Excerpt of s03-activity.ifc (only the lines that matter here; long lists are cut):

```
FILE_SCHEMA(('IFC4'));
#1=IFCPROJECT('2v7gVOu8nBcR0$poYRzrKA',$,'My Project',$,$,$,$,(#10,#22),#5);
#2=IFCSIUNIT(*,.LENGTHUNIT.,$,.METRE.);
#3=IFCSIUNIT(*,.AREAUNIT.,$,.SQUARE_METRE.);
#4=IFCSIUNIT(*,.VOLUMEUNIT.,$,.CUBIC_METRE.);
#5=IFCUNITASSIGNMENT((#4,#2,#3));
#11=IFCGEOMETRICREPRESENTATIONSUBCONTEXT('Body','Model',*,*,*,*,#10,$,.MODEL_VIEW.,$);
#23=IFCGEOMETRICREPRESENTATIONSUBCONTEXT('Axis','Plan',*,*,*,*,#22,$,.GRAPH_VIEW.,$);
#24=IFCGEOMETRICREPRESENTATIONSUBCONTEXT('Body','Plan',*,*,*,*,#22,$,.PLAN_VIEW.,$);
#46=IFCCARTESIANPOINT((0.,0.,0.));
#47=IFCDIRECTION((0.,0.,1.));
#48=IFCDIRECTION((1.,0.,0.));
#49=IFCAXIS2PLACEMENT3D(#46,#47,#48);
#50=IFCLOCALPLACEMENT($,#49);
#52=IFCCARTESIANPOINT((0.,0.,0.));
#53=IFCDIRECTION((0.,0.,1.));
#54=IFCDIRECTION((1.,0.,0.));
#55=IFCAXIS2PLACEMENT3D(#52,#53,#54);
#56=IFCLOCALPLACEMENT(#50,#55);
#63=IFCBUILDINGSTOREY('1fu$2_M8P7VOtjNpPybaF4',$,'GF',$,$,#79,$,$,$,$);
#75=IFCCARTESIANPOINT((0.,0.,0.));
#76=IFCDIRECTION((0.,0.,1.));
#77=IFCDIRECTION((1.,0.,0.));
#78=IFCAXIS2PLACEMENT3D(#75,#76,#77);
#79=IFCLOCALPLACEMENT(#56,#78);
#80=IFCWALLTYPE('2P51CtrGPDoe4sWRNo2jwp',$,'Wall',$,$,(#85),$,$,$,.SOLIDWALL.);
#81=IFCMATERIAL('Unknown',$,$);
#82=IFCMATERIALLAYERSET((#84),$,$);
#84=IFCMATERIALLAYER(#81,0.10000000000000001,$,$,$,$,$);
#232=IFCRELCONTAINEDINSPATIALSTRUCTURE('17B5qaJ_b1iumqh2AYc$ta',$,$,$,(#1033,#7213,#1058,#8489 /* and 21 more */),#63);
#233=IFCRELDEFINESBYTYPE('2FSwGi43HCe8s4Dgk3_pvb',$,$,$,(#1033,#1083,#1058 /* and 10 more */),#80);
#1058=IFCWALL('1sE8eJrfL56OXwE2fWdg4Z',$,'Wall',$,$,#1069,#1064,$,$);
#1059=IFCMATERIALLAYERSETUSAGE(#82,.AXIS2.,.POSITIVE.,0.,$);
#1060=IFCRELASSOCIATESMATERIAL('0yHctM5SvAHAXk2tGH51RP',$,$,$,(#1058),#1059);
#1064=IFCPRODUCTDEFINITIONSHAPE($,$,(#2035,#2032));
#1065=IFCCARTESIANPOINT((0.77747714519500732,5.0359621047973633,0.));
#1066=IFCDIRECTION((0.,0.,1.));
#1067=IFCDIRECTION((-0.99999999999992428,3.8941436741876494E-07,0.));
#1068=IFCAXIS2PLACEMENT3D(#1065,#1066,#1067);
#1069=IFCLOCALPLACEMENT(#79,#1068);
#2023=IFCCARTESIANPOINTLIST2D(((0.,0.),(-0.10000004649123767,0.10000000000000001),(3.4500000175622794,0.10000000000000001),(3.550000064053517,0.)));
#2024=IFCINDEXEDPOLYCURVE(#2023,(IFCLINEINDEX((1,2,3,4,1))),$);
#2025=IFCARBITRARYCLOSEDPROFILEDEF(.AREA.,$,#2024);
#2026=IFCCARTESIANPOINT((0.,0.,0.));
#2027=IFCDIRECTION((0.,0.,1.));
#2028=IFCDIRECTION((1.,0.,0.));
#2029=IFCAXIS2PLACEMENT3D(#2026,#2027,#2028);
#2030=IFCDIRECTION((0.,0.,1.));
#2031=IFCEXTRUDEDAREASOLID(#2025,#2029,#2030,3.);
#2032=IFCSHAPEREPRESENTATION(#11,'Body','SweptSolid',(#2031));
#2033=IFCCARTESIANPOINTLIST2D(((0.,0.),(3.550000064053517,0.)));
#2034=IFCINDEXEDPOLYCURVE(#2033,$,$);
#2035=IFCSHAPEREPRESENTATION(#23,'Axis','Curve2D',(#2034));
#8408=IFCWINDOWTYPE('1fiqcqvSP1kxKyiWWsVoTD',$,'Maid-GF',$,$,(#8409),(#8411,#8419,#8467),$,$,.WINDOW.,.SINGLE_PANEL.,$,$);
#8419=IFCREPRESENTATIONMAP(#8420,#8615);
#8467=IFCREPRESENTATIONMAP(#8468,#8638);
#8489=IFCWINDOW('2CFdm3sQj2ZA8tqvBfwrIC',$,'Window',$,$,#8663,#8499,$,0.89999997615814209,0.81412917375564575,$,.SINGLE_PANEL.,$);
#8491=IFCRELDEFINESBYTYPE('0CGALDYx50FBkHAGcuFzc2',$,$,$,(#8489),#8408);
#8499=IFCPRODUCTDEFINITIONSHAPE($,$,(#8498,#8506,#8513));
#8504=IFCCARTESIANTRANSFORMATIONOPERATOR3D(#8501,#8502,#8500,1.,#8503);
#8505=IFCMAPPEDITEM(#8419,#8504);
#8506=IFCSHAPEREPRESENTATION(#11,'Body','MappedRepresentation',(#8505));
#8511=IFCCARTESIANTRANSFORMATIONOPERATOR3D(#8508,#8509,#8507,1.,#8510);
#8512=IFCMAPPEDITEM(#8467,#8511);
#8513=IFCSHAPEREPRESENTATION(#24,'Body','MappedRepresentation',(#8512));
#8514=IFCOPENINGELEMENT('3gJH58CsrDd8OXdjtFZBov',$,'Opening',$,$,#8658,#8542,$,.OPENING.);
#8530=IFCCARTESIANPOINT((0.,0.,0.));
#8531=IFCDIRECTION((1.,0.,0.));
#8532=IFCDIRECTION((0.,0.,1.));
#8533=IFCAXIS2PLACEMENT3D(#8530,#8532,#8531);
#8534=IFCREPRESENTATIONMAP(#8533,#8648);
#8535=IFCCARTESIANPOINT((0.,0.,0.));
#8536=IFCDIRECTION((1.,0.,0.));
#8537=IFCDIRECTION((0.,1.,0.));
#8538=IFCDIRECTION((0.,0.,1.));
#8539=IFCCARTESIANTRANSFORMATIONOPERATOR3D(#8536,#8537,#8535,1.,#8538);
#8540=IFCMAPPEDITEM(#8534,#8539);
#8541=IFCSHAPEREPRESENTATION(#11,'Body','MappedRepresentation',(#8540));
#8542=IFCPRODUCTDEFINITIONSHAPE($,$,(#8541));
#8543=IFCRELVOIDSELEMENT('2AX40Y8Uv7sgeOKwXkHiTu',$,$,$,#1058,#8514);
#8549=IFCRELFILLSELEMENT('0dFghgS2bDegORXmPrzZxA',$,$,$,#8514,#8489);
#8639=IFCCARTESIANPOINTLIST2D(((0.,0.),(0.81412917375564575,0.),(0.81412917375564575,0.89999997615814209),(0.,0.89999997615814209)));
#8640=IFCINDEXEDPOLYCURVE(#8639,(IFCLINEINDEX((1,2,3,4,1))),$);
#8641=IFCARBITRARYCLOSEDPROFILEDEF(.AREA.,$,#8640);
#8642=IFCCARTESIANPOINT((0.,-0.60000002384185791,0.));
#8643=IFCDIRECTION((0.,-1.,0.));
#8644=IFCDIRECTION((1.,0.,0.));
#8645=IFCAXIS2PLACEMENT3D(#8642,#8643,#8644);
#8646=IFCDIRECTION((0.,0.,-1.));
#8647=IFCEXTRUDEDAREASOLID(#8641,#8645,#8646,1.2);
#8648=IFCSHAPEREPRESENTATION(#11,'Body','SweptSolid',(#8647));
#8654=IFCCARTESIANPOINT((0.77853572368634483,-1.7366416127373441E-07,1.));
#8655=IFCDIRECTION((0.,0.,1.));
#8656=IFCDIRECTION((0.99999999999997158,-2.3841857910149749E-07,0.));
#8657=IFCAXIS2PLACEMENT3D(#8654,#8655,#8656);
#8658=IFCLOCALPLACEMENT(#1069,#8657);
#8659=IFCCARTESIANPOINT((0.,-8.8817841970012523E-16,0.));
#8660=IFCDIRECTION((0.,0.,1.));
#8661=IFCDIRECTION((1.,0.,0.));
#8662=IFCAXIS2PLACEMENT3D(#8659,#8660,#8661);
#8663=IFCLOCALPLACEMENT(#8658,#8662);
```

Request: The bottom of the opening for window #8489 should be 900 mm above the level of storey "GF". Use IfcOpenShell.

```python
import numpy as np
import ifcopenshell
import ifcopenshell.api.geometry
import ifcopenshell.geom
import ifcopenshell.util.element
import ifcopenshell.util.placement
import ifcopenshell.util.shape
import ifcopenshell.util.unit

model = ifcopenshell.open("s03-activity.ifc")
unit_scale = ifcopenshell.util.unit.calculate_unit_scale(model)

window = model.by_guid("2CFdm3sQj2ZA8tqvBfwrIC")
opening = window.FillsVoids[0].RelatingOpeningElement
storey = ifcopenshell.util.element.get_container(window, ifc_class="IfcBuildingStorey")
level = ifcopenshell.util.placement.get_local_placement(storey.ObjectPlacement)[2, 3]

# The opening's origin need not be at the sill, so measure its lowest point.
shape = ifcopenshell.geom.create_shape(ifcopenshell.geom.settings(), opening)
bottom = ifcopenshell.util.shape.get_shape_bottom_elevation(shape, shape.geometry) / unit_scale
dz = level + 0.9 / unit_scale - bottom

shift = np.array([0.0, 0.0, dz])
# The window is placed relative to its opening, so it follows when the opening moves.
matrix = ifcopenshell.util.placement.get_local_placement(opening.ObjectPlacement)
matrix[:3, 3] += shift
ifcopenshell.api.geometry.edit_object_placement(
    model, product=opening, matrix=matrix, is_si=False, should_transform_children=True
)

print(f"moved by {dz * unit_scale:+.3f} m")

model.write("s03-activity_updated.ifc")
```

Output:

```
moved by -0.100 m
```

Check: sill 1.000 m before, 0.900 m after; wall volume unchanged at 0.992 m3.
